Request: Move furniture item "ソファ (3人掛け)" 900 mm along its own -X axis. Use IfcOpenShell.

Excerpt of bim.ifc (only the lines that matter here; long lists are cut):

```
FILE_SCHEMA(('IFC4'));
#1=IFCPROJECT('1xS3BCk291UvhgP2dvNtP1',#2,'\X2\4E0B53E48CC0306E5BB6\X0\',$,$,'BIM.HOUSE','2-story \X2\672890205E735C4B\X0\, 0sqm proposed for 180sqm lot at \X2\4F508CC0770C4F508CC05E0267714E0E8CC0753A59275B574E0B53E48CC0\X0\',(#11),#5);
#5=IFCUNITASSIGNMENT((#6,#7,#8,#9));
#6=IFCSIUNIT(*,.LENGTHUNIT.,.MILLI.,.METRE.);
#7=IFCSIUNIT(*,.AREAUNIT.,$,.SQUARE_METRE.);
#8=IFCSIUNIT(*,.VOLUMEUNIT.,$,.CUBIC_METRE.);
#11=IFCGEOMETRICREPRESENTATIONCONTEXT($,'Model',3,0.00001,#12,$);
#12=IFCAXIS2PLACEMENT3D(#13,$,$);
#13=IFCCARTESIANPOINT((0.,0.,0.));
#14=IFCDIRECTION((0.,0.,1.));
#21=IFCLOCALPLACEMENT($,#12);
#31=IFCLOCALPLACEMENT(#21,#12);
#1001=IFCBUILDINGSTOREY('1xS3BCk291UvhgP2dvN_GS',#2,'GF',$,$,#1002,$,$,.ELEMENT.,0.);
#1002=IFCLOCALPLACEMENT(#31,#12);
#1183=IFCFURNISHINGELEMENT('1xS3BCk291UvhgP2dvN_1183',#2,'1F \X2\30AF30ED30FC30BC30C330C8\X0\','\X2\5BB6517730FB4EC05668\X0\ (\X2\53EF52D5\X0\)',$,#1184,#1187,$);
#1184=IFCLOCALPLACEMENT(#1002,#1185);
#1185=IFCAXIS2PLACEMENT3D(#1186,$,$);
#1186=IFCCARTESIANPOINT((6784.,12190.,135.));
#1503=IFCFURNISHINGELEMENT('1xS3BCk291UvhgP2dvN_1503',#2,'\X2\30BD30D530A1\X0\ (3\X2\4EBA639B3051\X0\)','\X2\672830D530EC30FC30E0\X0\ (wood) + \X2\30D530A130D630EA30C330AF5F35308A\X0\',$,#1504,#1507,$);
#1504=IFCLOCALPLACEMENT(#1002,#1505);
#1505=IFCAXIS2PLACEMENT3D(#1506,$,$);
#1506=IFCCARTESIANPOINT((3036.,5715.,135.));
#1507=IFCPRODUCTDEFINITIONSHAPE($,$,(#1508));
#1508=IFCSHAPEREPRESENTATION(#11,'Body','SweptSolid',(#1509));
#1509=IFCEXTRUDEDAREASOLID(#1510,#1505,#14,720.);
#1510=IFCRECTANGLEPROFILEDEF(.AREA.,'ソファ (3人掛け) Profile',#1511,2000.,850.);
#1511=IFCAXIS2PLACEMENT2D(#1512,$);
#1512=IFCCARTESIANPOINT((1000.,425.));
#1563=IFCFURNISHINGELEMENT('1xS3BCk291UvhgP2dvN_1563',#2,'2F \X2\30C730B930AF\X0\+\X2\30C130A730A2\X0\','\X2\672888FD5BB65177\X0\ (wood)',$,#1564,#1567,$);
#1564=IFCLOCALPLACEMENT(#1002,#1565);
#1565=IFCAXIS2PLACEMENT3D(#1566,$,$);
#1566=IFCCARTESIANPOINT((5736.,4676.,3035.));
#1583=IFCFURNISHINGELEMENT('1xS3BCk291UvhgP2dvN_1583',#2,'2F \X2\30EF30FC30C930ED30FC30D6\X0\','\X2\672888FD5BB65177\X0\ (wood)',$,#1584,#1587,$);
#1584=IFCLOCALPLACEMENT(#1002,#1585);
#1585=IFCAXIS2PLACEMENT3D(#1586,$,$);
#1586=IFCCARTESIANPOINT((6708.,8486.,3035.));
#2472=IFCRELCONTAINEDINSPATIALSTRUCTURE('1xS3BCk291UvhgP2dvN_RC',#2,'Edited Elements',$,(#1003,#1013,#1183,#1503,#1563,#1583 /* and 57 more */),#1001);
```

```python
import ifcopenshell
import ifcopenshell.api.geometry
import ifcopenshell.util.placement
import ifcopenshell.util.unit

model = ifcopenshell.open("bim.ifc")
unit_scale = ifcopenshell.util.unit.calculate_unit_scale(model)

item = model.by_id(1503)
matrix = ifcopenshell.util.placement.get_local_placement(item.ObjectPlacement)
matrix[:3, 3] -= matrix[:3, 0] * 0.9 / unit_scale
ifcopenshell.api.geometry.edit_object_placement(model, product=item, matrix=matrix, is_si=False)

print(ifcopenshell.util.placement.get_local_placement(item.ObjectPlacement).round(3) + 0.0)

model.write("bim_edited.ifc")
```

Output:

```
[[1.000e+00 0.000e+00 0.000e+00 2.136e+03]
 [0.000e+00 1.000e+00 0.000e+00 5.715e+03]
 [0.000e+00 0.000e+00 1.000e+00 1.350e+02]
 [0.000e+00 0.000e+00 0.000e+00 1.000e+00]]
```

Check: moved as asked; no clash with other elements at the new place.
